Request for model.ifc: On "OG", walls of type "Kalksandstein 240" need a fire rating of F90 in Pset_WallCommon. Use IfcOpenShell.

First a look at what the model holds.

```python
import ifcopenshell
import ifcopenshell.util.element

model = ifcopenshell.open("model.ifc")
print(model.schema)
storey = next(s for s in model.by_type("IfcBuildingStorey") if s.Name == "OG")
walls = [e for e in ifcopenshell.util.element.get_decomposition(storey) if e.is_a("IfcWall")]
seen = {}
for e in walls:
    element_type = ifcopenshell.util.element.get_type(e)
    key = (element_type.Name if element_type != e and element_type else None, ifcopenshell.util.element.get_pset(e, "Pset_WallCommon", "FireRating"))
    seen[key] = seen.get(key, 0) + 1
for (name, value), count in sorted(seen.items(), key=str):
    print(count, "x", name, "|", value)
```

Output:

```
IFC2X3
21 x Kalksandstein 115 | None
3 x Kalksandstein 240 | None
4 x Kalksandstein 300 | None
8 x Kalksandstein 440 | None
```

```python
import ifcopenshell
import ifcopenshell.api.pset
import ifcopenshell.util.element

model = ifcopenshell.open("model.ifc")

storey = next(s for s in model.by_type("IfcBuildingStorey") if s.Name == "OG")
walls = [e for e in ifcopenshell.util.element.get_decomposition(storey) if e.is_a("IfcWall")]

count = 0
for e in walls:
    element_type = ifcopenshell.util.element.get_type(e)
    if element_type in (None, e) or element_type.Name != "Kalksandstein 240":
        continue
    # add_pset returns the element's existing set when there is one.
    pset = ifcopenshell.api.pset.add_pset(model, product=e, name="Pset_WallCommon")
    ifcopenshell.api.pset.edit_pset(model, pset=pset, properties={"FireRating": "F90"})
    count += 1

print(count, "walls updated")

model.write("model_rev.ifc")
```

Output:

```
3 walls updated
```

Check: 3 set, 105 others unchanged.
